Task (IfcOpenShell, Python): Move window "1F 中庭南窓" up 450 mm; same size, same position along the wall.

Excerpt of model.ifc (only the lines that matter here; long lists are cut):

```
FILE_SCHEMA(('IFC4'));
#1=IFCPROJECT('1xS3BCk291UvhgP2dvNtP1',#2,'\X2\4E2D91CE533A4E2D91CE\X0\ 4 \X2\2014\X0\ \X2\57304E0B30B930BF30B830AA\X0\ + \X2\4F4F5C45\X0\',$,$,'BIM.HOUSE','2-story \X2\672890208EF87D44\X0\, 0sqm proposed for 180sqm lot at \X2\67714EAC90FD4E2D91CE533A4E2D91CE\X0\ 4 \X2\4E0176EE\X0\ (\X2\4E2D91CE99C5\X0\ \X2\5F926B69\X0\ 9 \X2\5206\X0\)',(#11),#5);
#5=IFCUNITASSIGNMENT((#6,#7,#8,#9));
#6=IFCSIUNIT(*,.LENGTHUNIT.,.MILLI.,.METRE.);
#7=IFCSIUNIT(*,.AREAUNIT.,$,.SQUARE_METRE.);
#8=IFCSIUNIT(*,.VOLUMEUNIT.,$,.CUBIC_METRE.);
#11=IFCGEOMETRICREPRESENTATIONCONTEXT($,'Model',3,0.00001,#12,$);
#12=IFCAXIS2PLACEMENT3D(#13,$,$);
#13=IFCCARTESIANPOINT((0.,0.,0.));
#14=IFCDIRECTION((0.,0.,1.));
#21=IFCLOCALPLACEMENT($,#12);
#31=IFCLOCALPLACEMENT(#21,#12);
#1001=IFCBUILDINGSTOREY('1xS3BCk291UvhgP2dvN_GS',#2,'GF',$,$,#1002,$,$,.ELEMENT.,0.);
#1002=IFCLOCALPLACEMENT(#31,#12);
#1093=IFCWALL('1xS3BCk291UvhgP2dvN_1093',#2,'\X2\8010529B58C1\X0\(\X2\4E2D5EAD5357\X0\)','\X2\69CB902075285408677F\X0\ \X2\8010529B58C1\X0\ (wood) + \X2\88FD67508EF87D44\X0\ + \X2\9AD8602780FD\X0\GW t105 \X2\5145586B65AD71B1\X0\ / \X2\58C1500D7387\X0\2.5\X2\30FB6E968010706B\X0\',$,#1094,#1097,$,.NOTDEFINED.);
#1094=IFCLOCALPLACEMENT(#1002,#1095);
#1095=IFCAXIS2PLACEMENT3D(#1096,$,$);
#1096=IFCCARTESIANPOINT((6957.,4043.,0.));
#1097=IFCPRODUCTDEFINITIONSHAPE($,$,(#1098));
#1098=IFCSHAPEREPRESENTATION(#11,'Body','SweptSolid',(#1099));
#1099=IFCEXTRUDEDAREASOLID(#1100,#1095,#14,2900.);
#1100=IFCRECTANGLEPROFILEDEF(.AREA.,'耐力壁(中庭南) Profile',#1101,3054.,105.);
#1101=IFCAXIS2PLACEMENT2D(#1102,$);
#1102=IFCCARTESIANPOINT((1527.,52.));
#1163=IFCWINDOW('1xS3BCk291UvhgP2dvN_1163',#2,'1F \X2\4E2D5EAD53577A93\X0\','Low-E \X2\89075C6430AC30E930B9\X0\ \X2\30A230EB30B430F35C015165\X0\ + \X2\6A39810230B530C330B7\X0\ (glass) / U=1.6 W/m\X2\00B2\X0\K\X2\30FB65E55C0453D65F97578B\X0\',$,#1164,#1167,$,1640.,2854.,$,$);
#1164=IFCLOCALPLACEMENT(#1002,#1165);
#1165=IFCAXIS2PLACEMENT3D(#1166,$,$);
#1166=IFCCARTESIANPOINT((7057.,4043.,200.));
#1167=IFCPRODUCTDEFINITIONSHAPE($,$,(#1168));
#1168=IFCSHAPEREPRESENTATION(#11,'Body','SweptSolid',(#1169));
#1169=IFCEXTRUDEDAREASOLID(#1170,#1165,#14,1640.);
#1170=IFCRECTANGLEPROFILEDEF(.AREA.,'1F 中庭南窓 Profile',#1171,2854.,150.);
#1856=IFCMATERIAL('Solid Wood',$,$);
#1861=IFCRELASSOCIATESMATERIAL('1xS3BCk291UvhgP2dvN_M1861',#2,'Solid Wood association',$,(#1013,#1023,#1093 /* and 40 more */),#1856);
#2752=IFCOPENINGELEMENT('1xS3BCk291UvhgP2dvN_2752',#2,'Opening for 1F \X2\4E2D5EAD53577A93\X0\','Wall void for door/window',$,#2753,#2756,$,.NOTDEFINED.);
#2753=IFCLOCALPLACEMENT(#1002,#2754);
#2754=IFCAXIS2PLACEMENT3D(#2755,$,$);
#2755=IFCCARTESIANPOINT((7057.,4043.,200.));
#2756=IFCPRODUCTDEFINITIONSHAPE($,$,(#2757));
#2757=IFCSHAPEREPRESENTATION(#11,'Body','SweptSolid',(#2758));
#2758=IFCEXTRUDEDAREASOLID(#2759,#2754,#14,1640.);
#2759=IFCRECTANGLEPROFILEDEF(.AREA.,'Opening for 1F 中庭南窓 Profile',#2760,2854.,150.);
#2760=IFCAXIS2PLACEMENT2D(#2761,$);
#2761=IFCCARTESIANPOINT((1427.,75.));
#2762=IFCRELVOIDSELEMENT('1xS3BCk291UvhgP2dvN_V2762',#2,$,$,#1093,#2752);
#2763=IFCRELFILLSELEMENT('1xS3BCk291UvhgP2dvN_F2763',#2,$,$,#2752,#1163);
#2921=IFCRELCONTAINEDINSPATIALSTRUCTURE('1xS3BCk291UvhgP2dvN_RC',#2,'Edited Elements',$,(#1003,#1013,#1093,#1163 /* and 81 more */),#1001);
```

```python
import numpy as np
import ifcopenshell
import ifcopenshell.api.geometry
import ifcopenshell.util.placement
import ifcopenshell.util.unit

model = ifcopenshell.open("model.ifc")
unit_scale = ifcopenshell.util.unit.calculate_unit_scale(model)

window = model.by_guid("1xS3BCk291UvhgP2dvN_1163")
opening = window.FillsVoids[0].RelatingOpeningElement
dz = 450.0

shift = np.array([0.0, 0.0, dz])
# The window is not placed relative to its opening, so move both.
for product in (opening, window):
    matrix = ifcopenshell.util.placement.get_local_placement(product.ObjectPlacement)
    matrix[:3, 3] += shift
    ifcopenshell.api.geometry.edit_object_placement(model, product=product, matrix=matrix, is_si=False)

print(f"moved by {dz * unit_scale:+.3f} m")

model.write("model_edited.ifc")
```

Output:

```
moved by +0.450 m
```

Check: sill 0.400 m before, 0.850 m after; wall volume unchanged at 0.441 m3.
